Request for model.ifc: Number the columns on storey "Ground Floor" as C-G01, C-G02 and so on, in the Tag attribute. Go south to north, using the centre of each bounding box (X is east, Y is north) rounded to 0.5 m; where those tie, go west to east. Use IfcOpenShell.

First a look at what the model holds.

```python
import ifcopenshell
import ifcopenshell.util.element
import ifcopenshell.util.placement

model = ifcopenshell.open("model.ifc")
print(model.schema)
storey = next(s for s in model.by_type("IfcBuildingStorey") if s.Name == "Ground Floor")
columns = [e for e in ifcopenshell.util.element.get_decomposition(storey) if e.is_a("IfcColumn")]
for e in sorted(columns, key=lambda e: e.id()):
    origin = ifcopenshell.util.placement.get_local_placement(e.ObjectPlacement)[:3, 3]
    print(e.id(), e.Tag, e.Name, origin.round(2) + 0.0, sep=" | ")
```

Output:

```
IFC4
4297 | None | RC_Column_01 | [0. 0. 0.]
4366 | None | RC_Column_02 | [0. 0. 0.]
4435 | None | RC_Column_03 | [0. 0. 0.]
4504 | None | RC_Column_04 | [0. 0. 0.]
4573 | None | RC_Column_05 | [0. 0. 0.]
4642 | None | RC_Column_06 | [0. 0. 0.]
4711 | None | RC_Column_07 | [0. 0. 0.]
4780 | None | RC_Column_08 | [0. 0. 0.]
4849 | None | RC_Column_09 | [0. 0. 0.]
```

```python
import ifcopenshell
import ifcopenshell.geom
import ifcopenshell.util.element
import ifcopenshell.util.shape

model = ifcopenshell.open("model.ifc")
settings = ifcopenshell.geom.settings()
settings.set("use-world-coords", True)


def centre(element):
    shape = ifcopenshell.geom.create_shape(settings, element)
    return ifcopenshell.util.shape.get_bbox_centroid(shape.geometry)


storey = next(s for s in model.by_type("IfcBuildingStorey") if s.Name == "Ground Floor")
columns = [e for e in ifcopenshell.util.element.get_decomposition(storey) if e.is_a("IfcColumn")]

# Insertion points can sit at a corner or the storey origin, so sort by the geometry (in metres).
centres = {e: centre(e) for e in columns}
columns.sort(key=lambda e: (round(centres[e][1] / 0.5), centres[e][0]))

for i, e in enumerate(columns, start=1):
    number = f"C-G{i:02d}"
    e.Tag = number
    print(e.id(), number)

model.write("model-out.ifc")
```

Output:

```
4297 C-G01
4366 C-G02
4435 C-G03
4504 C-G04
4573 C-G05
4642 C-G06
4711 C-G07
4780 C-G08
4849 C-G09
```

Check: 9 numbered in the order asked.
